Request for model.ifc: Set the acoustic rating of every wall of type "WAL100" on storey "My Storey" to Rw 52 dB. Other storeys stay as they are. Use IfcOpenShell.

First a look at what the model holds.

```python
import ifcopenshell
import ifcopenshell.util.element

model = ifcopenshell.open("model.ifc")
print(model.schema)
storey = next(s for s in model.by_type("IfcBuildingStorey") if s.Name == "My Storey")
walls = [e for e in ifcopenshell.util.element.get_decomposition(storey) if e.is_a("IfcWall")]
seen = {}
for e in walls:
    element_type = ifcopenshell.util.element.get_type(e)
    key = (element_type.Name if element_type != e and element_type else None, ifcopenshell.util.element.get_pset(e, "Pset_WallCommon", "AcousticRating"))
    seen[key] = seen.get(key, 0) + 1
for (name, value), count in sorted(seen.items(), key=str):
    print(count, "x", name, "|", value)
```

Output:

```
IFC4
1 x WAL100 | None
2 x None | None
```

```python
import ifcopenshell
import ifcopenshell.api.pset
import ifcopenshell.util.element

model = ifcopenshell.open("model.ifc")

storey = next(s for s in model.by_type("IfcBuildingStorey") if s.Name == "My Storey")
walls = [e for e in ifcopenshell.util.element.get_decomposition(storey) if e.is_a("IfcWall")]

count = 0
for e in walls:
    element_type = ifcopenshell.util.element.get_type(e)
    if element_type in (None, e) or element_type.Name != "WAL100":
        continue
    # add_pset returns the element's existing set when there is one.
    pset = ifcopenshell.api.pset.add_pset(model, product=e, name="Pset_WallCommon")
    ifcopenshell.api.pset.edit_pset(model, pset=pset, properties={"AcousticRating": "Rw 52 dB"})
    count += 1

print(count, "walls updated")

model.write("model_rev.ifc")
```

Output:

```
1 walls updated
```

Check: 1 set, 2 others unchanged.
